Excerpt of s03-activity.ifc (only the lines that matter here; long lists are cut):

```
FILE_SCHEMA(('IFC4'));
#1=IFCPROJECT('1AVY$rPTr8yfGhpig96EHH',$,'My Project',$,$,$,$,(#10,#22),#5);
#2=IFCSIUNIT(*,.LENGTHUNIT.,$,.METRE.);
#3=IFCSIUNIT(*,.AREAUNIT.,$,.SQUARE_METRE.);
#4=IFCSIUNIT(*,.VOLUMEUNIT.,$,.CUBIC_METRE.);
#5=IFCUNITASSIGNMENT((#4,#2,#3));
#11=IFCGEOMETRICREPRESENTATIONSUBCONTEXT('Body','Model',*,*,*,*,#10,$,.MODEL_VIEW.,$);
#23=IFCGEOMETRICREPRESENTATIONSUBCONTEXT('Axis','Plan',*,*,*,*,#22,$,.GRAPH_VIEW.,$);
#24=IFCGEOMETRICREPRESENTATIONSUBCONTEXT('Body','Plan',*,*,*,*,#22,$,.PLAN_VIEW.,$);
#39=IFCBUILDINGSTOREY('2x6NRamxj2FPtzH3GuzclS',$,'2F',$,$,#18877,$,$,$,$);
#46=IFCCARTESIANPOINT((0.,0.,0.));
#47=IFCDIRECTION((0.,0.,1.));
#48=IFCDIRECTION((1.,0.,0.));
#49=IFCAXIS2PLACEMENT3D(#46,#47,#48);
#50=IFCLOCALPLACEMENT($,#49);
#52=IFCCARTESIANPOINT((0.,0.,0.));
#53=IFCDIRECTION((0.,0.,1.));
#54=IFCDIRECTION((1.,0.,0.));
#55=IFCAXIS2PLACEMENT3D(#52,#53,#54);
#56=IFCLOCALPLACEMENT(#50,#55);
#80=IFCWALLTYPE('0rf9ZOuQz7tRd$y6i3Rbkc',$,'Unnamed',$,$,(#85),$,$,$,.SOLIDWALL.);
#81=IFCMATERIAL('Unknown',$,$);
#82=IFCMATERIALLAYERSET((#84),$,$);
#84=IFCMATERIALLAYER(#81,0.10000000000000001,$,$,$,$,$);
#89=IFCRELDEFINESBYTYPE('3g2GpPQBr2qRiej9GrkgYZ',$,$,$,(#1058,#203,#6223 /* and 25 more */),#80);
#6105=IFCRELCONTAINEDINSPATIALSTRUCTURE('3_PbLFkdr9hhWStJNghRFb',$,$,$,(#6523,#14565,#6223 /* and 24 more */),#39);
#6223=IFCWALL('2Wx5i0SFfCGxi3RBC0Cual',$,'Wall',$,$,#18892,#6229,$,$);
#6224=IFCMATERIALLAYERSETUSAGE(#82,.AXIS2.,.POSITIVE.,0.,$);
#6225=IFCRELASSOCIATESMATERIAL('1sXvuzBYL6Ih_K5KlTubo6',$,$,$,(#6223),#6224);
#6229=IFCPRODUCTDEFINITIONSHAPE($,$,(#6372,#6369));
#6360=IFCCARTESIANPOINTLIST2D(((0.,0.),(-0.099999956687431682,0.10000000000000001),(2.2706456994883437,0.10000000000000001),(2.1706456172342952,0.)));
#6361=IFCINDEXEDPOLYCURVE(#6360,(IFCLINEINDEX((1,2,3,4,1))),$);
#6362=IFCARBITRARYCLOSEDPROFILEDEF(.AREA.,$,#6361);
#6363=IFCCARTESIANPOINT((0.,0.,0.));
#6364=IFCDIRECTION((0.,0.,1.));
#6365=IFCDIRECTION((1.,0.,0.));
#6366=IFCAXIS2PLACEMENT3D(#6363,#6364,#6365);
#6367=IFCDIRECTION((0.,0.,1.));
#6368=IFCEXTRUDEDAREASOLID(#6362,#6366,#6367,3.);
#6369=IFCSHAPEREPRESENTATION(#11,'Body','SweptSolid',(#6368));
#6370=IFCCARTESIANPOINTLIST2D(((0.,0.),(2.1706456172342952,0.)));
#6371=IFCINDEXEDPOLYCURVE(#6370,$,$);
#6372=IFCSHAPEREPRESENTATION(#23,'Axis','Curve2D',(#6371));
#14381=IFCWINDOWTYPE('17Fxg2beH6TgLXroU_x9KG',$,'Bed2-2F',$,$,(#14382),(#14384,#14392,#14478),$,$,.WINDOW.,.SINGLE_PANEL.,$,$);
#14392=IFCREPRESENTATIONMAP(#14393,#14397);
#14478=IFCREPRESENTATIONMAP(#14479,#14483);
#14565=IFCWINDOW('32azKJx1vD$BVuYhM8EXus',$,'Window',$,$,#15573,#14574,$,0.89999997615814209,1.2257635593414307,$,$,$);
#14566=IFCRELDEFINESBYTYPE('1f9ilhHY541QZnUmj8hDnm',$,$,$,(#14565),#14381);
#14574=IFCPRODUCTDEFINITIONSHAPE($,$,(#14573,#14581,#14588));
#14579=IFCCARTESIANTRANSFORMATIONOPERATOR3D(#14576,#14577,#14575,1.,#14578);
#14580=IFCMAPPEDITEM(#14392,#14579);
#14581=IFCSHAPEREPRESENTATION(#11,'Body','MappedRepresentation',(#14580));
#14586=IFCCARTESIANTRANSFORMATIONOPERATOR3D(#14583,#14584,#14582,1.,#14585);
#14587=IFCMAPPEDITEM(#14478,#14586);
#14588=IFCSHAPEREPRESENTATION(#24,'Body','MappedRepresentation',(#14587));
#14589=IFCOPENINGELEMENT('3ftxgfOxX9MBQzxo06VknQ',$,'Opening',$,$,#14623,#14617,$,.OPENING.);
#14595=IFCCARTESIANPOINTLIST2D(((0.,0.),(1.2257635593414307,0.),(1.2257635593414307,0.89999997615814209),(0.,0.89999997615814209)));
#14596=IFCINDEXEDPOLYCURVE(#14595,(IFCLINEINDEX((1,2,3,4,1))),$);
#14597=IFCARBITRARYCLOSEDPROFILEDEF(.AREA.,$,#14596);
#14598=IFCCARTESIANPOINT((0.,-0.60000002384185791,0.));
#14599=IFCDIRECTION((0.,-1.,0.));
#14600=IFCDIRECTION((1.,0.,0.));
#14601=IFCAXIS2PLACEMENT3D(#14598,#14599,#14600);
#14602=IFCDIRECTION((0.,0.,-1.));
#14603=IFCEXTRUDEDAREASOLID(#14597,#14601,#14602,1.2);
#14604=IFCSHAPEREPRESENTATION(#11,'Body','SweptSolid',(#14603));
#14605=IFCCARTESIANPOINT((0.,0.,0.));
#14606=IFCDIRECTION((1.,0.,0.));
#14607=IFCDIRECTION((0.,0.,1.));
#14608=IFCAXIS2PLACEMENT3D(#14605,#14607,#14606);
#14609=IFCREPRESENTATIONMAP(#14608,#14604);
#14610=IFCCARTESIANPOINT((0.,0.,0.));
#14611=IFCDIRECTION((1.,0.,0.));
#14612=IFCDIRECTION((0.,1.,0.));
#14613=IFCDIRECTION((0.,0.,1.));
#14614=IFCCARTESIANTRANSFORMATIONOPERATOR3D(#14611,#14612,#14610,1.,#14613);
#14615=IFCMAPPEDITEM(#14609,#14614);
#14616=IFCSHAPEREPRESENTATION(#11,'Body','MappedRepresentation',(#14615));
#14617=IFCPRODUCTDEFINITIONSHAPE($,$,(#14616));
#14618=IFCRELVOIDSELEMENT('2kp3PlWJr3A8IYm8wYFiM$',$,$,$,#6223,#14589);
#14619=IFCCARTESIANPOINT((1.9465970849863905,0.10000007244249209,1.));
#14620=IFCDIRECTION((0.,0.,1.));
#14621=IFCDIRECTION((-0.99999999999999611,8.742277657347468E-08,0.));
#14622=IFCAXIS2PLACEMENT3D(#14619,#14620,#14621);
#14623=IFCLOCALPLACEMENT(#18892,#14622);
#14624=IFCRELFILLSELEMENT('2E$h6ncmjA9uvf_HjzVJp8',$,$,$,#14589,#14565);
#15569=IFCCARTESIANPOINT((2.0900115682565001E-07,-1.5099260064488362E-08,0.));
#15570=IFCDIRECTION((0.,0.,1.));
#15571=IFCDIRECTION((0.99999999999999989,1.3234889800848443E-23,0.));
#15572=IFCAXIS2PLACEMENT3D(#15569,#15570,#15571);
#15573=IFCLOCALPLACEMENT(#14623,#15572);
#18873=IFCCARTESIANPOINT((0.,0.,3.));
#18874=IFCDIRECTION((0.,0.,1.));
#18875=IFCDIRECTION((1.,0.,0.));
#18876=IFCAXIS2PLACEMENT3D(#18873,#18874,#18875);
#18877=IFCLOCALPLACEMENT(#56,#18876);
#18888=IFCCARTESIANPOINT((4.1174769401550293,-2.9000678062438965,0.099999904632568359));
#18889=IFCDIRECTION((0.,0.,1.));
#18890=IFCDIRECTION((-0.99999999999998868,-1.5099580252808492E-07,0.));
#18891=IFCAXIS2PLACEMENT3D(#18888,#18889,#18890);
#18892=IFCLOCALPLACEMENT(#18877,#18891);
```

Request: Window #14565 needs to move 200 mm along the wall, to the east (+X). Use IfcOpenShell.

```python
import ifcopenshell
import ifcopenshell.api.geometry
import ifcopenshell.util.placement

model = ifcopenshell.open("s03-activity.ifc")

window = model.by_guid("32azKJx1vD$BVuYhM8EXus")
opening = window.FillsVoids[0].RelatingOpeningElement
wall = opening.VoidsElements[0].RelatingBuildingElement

wall_matrix = ifcopenshell.util.placement.get_local_placement(wall.ObjectPlacement)
shift = wall_matrix[:3, 0] * -0.2
before = ifcopenshell.util.placement.get_local_placement(window.ObjectPlacement)[:3, 3].copy()

# The window is placed relative to its opening, so it follows when the opening moves.
matrix = ifcopenshell.util.placement.get_local_placement(opening.ObjectPlacement)
matrix[:3, 3] += shift
ifcopenshell.api.geometry.edit_object_placement(
    model, product=opening, matrix=matrix, is_si=False, should_transform_children=True
)

after = ifcopenshell.util.placement.get_local_placement(window.ObjectPlacement)[:3, 3]
print("window moved by", (after - before).round(3) + 0.0)

model.write("s03-activity_updated.ifc")
```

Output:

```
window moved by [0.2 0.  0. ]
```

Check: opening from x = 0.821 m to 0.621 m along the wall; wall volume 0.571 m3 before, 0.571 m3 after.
